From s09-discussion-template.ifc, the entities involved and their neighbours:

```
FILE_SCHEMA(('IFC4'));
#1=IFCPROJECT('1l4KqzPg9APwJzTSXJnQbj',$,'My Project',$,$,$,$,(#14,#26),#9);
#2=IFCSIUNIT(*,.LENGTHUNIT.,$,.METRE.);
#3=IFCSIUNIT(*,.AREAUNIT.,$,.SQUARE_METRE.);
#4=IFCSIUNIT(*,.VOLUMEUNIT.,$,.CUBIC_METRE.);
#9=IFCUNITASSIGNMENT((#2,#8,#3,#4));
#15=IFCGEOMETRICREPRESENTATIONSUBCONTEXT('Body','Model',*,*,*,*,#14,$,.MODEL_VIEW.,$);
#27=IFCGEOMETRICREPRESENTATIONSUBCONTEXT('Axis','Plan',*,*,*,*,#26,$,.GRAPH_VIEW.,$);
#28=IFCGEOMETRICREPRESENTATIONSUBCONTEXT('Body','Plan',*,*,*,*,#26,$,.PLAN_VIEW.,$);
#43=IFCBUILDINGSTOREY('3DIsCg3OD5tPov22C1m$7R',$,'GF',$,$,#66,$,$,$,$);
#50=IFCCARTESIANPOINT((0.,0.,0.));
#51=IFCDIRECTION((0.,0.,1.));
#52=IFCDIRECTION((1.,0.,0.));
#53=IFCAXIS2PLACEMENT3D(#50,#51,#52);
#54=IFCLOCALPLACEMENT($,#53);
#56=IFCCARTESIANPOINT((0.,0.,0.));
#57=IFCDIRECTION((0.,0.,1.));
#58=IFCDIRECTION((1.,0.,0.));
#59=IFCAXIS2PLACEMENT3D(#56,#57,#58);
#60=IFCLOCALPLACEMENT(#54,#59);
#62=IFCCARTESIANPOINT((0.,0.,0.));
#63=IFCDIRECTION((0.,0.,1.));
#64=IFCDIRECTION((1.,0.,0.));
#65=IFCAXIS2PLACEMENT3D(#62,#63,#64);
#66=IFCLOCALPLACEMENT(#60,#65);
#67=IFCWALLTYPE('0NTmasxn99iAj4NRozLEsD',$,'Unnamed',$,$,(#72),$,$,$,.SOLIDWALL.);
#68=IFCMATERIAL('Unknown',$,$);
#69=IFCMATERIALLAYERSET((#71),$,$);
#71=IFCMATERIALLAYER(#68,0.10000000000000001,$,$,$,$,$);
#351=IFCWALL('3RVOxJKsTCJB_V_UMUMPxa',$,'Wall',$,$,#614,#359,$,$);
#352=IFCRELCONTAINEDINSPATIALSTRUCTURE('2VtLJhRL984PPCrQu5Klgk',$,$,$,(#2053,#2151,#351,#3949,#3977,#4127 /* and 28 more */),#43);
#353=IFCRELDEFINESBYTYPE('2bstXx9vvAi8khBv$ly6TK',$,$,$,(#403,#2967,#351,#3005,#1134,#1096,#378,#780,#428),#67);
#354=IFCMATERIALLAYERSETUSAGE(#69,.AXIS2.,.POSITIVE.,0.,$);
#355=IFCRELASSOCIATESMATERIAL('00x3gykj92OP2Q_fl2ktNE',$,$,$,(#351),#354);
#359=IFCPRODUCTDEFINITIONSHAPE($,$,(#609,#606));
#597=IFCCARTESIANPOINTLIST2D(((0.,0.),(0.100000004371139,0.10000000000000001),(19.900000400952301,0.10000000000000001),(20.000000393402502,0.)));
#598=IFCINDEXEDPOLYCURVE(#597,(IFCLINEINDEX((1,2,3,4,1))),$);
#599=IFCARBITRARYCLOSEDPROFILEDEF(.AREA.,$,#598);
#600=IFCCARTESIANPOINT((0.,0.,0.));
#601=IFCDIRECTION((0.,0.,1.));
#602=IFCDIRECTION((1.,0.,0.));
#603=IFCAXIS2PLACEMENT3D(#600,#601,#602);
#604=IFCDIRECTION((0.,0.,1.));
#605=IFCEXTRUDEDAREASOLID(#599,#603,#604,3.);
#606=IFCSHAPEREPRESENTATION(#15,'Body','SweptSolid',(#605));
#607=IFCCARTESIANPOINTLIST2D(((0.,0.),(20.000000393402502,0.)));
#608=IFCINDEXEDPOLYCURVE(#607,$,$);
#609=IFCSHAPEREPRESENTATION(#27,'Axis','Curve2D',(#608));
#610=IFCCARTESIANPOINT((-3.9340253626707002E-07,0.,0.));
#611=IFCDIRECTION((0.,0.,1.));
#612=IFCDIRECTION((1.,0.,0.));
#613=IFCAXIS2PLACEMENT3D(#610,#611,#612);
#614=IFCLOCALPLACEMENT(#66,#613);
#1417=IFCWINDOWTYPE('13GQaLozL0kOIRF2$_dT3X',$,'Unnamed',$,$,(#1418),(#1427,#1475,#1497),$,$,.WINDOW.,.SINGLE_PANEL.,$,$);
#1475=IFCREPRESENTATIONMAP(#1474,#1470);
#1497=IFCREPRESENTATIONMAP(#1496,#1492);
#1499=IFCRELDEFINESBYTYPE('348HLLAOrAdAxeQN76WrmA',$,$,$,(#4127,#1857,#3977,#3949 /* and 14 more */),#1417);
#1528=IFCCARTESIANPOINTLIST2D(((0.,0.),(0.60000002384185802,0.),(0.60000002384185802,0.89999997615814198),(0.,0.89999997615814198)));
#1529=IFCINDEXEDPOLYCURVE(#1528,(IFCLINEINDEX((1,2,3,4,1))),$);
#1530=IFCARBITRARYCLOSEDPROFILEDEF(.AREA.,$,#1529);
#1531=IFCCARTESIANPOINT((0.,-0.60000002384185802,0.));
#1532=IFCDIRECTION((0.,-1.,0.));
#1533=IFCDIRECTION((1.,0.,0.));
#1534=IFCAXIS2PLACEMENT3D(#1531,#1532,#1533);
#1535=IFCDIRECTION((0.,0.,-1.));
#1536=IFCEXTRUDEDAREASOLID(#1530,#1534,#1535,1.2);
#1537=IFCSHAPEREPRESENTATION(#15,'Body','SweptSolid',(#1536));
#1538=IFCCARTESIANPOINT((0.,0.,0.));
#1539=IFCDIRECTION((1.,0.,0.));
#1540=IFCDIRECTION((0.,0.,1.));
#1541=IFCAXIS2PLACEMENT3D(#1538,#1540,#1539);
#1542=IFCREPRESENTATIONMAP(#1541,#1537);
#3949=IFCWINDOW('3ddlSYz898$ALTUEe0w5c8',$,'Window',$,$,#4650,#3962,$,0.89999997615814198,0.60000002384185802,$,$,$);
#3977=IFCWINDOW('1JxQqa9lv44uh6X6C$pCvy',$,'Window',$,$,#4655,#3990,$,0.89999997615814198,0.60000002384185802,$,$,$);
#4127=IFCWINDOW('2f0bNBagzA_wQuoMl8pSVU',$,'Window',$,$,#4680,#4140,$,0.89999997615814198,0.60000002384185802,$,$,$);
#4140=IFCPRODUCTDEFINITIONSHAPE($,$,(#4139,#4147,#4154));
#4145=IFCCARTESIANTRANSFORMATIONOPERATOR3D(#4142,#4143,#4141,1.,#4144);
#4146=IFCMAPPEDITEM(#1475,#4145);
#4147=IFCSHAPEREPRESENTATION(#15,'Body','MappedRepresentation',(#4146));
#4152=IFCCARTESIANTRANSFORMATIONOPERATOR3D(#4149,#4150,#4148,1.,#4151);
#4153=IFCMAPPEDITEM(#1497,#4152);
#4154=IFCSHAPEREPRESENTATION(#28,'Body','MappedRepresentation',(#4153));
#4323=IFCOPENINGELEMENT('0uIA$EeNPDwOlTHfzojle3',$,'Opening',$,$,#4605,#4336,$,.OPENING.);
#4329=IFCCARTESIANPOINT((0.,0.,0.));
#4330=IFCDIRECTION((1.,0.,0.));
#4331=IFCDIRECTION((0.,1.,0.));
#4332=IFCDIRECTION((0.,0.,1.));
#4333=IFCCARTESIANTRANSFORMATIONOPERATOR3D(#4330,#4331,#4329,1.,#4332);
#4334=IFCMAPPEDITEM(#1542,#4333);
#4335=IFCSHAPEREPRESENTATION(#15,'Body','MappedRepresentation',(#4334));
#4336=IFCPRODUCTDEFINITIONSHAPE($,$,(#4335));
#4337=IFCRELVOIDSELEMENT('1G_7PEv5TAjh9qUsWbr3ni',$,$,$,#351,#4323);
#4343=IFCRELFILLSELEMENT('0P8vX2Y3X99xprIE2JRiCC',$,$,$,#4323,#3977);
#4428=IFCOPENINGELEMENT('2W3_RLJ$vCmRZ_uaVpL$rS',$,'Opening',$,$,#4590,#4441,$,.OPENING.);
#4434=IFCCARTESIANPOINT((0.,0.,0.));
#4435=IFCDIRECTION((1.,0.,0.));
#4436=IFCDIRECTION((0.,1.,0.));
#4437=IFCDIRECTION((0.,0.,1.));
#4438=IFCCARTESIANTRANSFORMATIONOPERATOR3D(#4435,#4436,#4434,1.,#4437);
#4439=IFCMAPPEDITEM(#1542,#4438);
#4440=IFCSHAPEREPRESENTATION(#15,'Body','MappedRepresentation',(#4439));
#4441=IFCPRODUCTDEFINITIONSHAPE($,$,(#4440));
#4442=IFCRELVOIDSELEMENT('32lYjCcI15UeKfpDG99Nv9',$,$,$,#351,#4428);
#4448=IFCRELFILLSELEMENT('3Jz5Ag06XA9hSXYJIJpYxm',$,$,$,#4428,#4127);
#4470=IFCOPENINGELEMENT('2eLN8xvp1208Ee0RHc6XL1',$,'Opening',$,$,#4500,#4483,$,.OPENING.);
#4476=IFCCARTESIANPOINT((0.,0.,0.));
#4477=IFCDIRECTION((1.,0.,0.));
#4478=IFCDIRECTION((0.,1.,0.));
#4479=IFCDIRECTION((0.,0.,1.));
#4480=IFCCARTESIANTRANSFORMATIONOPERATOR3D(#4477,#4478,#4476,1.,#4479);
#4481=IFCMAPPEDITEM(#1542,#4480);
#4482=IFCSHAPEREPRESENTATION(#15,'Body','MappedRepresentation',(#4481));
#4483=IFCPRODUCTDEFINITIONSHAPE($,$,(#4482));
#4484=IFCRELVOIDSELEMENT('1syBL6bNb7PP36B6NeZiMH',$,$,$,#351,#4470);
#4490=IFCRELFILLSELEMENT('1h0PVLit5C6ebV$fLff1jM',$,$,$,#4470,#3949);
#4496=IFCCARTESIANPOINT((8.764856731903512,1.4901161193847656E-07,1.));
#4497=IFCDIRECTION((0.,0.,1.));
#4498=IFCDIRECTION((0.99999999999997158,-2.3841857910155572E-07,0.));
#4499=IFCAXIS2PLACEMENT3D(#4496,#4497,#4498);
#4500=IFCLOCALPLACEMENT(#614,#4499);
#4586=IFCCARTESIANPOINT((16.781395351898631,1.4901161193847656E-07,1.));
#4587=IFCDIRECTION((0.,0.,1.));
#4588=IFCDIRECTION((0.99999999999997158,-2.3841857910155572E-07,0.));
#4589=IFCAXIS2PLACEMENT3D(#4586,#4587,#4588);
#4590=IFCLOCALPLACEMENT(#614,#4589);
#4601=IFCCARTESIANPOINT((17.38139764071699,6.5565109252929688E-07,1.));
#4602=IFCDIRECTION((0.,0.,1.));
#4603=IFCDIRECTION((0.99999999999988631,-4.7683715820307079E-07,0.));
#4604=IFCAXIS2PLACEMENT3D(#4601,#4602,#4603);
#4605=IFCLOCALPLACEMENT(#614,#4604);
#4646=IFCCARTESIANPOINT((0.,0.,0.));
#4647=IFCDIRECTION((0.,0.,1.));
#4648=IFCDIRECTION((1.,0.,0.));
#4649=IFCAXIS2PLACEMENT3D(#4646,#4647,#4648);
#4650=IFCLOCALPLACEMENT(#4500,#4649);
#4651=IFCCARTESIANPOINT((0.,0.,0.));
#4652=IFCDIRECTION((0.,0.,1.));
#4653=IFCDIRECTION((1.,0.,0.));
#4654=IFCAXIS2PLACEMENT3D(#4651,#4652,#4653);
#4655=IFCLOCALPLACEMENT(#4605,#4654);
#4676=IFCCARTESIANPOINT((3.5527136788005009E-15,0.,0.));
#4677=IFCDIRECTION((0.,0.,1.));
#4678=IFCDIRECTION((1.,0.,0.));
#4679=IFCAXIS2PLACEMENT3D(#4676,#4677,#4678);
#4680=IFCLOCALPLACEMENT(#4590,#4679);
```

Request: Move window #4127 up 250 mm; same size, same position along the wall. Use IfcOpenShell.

```python
import numpy as np
import ifcopenshell
import ifcopenshell.api.geometry
import ifcopenshell.util.placement
import ifcopenshell.util.unit

model = ifcopenshell.open("s09-discussion-template.ifc")
unit_scale = ifcopenshell.util.unit.calculate_unit_scale(model)

window = model.by_guid("2f0bNBagzA_wQuoMl8pSVU")
opening = window.FillsVoids[0].RelatingOpeningElement
dz = 0.25 / unit_scale

shift = np.array([0.0, 0.0, dz])
# The window is placed relative to its opening, so it follows when the opening moves.
matrix = ifcopenshell.util.placement.get_local_placement(opening.ObjectPlacement)
matrix[:3, 3] += shift
ifcopenshell.api.geometry.edit_object_placement(
    model, product=opening, matrix=matrix, is_si=False, should_transform_children=True
)

print(f"moved by {dz * unit_scale:+.3f} m")

model.write("s09-discussion-template_updated.ifc")
```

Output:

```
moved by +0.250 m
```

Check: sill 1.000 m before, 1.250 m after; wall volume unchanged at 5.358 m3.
